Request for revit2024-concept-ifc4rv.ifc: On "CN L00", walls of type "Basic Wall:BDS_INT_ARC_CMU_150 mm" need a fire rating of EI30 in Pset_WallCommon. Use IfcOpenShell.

First a look at what the model holds.

```python
import ifcopenshell
import ifcopenshell.util.element

model = ifcopenshell.open("revit2024-concept-ifc4rv.ifc")
print(model.schema)
storey = next(s for s in model.by_type("IfcBuildingStorey") if s.Name == "CN L00")
walls = [e for e in ifcopenshell.util.element.get_decomposition(storey) if e.is_a("IfcWall")]
seen = {}
for e in walls:
    element_type = ifcopenshell.util.element.get_type(e)
    key = (element_type.Name if element_type != e and element_type else None, ifcopenshell.util.element.get_pset(e, "Pset_WallCommon", "FireRating"))
    seen[key] = seen.get(key, 0) + 1
for (name, value), count in sorted(seen.items(), key=str):
    print(count, "x", name, "|", value)
```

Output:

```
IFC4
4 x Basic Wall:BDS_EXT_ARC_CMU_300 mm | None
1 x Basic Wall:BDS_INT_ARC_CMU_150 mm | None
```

```python
import ifcopenshell
import ifcopenshell.api.pset
import ifcopenshell.util.element

model = ifcopenshell.open("revit2024-concept-ifc4rv.ifc")

storey = next(s for s in model.by_type("IfcBuildingStorey") if s.Name == "CN L00")
walls = [e for e in ifcopenshell.util.element.get_decomposition(storey) if e.is_a("IfcWall")]

count = 0
for e in walls:
    element_type = ifcopenshell.util.element.get_type(e)
    if element_type in (None, e) or element_type.Name != "Basic Wall:BDS_INT_ARC_CMU_150 mm":
        continue
    # add_pset returns the element's existing set when there is one.
    pset = ifcopenshell.api.pset.add_pset(model, product=e, name="Pset_WallCommon")
    ifcopenshell.api.pset.edit_pset(model, pset=pset, properties={"FireRating": "EI30"})
    count += 1

print(count, "walls updated")

model.write("revit2024-concept-ifc4rv_edited.ifc")
```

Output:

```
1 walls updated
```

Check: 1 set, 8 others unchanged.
